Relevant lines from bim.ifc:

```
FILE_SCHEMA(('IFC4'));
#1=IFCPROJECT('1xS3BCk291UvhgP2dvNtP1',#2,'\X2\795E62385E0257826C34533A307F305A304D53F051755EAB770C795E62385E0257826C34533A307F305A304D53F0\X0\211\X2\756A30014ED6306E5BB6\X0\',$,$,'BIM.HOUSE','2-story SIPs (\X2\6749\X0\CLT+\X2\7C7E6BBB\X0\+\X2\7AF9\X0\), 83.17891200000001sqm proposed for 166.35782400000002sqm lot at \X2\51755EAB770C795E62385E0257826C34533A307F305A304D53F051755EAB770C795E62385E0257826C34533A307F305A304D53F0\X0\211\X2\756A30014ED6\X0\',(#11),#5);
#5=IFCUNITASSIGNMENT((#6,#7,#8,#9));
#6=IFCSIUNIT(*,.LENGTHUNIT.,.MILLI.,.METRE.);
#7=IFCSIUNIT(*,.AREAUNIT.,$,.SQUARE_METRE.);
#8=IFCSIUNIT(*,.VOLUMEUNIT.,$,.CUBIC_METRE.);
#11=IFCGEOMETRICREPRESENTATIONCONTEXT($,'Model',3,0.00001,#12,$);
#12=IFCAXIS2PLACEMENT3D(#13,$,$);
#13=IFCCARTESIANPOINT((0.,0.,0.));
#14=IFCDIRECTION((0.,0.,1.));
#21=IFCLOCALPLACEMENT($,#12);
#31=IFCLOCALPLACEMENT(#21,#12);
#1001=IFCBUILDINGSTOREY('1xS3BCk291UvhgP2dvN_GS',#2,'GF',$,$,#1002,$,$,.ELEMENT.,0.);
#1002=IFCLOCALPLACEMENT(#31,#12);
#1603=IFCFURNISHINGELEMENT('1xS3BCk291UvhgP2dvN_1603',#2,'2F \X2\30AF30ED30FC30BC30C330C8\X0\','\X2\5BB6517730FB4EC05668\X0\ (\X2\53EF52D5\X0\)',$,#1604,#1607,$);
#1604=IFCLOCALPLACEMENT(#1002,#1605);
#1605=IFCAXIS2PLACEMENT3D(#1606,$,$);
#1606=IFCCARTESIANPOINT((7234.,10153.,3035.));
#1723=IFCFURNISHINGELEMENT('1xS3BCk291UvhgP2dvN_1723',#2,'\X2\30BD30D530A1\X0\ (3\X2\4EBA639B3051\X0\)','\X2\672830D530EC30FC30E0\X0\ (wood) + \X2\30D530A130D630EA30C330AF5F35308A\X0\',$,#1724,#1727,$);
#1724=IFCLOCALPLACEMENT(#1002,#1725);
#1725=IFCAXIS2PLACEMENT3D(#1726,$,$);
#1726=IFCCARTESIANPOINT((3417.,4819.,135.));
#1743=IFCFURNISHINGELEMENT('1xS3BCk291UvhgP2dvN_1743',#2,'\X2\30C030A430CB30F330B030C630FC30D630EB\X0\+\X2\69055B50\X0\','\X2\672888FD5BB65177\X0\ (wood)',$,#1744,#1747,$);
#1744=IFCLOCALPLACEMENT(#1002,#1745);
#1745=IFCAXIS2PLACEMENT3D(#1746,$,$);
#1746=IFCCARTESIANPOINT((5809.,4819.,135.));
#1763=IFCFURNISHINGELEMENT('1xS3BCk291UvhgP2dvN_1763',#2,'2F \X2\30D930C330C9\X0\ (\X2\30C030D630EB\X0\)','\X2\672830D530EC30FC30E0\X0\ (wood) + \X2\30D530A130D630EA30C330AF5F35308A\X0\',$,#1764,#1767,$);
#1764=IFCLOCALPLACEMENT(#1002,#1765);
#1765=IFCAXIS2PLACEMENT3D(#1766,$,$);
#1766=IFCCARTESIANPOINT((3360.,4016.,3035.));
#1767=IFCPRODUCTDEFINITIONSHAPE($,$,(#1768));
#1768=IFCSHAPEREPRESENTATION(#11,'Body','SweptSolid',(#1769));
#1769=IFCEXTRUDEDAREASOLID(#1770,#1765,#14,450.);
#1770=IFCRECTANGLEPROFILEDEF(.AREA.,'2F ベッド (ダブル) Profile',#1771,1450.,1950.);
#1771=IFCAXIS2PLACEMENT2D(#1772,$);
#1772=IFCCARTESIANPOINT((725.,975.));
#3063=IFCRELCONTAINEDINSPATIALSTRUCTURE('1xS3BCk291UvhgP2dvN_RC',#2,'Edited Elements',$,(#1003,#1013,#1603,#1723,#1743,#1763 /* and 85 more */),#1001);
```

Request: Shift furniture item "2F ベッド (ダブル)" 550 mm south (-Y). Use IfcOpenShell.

```python
import ifcopenshell
import ifcopenshell.api.geometry
import ifcopenshell.util.placement
import ifcopenshell.util.unit

model = ifcopenshell.open("bim.ifc")
unit_scale = ifcopenshell.util.unit.calculate_unit_scale(model)

item = model.by_guid("1xS3BCk291UvhgP2dvN_1763")
matrix = ifcopenshell.util.placement.get_local_placement(item.ObjectPlacement)
matrix[1, 3] -= 0.55 / unit_scale
ifcopenshell.api.geometry.edit_object_placement(model, product=item, matrix=matrix, is_si=False)

print(ifcopenshell.util.placement.get_local_placement(item.ObjectPlacement).round(3) + 0.0)

model.write("bim_rev.ifc")
```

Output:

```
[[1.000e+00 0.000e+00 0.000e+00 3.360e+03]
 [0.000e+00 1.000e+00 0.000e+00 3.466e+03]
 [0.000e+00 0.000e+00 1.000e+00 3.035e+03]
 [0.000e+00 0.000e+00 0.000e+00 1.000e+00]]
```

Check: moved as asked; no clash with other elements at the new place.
